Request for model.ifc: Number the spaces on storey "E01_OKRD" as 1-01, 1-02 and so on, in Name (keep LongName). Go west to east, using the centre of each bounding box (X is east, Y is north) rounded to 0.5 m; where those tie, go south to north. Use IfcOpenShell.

First a look at what the model holds.

```python
import ifcopenshell
import ifcopenshell.util.element
import ifcopenshell.util.placement

model = ifcopenshell.open("model.ifc")
print(model.schema)
storey = next(s for s in model.by_type("IfcBuildingStorey") if s.Name == "E01_OKRD")
spaces = [e for e in ifcopenshell.util.element.get_decomposition(storey) if e.is_a("IfcSpace")]
for e in sorted(spaces, key=lambda e: e.id()):
    origin = ifcopenshell.util.placement.get_local_placement(e.ObjectPlacement)[:3, 3]
    print(e.id(), e.Name, e.LongName, origin.round(2) + 0.0, sep=" | ")
```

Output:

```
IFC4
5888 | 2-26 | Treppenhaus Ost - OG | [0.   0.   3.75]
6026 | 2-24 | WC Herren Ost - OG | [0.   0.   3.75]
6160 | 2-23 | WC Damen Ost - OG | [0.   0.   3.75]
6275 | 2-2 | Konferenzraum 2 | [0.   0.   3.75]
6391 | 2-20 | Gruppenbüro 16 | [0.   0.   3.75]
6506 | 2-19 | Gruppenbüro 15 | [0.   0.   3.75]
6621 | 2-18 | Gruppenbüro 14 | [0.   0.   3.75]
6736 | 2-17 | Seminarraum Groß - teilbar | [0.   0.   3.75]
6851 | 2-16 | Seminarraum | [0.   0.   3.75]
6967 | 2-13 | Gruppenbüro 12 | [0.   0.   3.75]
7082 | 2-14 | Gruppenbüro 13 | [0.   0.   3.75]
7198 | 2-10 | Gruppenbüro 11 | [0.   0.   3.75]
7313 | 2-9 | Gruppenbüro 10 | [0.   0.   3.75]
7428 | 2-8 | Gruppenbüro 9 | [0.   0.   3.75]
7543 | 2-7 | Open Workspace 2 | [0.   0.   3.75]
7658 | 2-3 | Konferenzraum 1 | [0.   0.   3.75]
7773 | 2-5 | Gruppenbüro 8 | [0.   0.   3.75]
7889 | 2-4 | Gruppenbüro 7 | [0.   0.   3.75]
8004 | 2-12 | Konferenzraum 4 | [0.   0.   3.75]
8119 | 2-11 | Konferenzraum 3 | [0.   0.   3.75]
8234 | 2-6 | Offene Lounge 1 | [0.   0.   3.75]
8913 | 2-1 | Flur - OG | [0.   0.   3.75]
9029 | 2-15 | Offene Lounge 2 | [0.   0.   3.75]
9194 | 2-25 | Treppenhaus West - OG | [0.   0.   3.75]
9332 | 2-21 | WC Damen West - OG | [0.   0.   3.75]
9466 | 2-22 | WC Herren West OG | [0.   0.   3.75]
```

```python
import ifcopenshell
import ifcopenshell.geom
import ifcopenshell.util.element
import ifcopenshell.util.shape

model = ifcopenshell.open("model.ifc")
settings = ifcopenshell.geom.settings()
settings.set("use-world-coords", True)


def centre(element):
    shape = ifcopenshell.geom.create_shape(settings, element)
    return ifcopenshell.util.shape.get_bbox_centroid(shape.geometry)


storey = next(s for s in model.by_type("IfcBuildingStorey") if s.Name == "E01_OKRD")
spaces = [e for e in ifcopenshell.util.element.get_decomposition(storey) if e.is_a("IfcSpace")]

# Insertion points can sit at a corner or the storey origin, so sort by the geometry (in metres).
centres = {e: centre(e) for e in spaces}
spaces.sort(key=lambda e: (round(centres[e][0] / 0.5), centres[e][1]))

for i, e in enumerate(spaces, start=1):
    number = f"1-{i:02d}"
    e.Name = number
    print(e.id(), number)

model.write("model_edited.ifc")
```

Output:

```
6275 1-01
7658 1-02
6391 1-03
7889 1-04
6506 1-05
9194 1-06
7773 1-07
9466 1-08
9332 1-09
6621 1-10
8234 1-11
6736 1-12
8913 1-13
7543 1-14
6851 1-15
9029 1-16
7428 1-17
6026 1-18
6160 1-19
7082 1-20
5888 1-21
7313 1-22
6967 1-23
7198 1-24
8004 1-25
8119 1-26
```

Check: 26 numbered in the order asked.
